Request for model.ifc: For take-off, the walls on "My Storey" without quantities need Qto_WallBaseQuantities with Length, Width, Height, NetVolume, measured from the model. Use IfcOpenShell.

First a look at what the model holds.

```python
import ifcopenshell
import ifcopenshell.util.element
import ifcopenshell.util.unit

model = ifcopenshell.open("model.ifc")
print(model.schema)
for unit_type in ("LENGTHUNIT", "AREAUNIT", "VOLUMEUNIT"):
    print(unit_type, ifcopenshell.util.unit.calculate_unit_scale(model, unit_type))
storey = next(s for s in model.by_type("IfcBuildingStorey") if s.Name == "My Storey")
walls = [e for e in ifcopenshell.util.element.get_decomposition(storey) if e.is_a("IfcWall")]
for e in sorted(walls, key=lambda e: e.id()):
    print(e.id(), e.is_a(), e.Name, list(ifcopenshell.util.element.get_psets(e, qtos_only=True)), sep=" | ")
```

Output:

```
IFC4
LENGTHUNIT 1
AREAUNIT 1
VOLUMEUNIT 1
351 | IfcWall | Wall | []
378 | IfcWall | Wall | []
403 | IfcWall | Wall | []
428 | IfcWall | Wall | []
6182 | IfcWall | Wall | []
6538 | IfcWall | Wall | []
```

```python
import ifcopenshell
import ifcopenshell.api.pset
import ifcopenshell.geom
import ifcopenshell.util.element
import ifcopenshell.util.shape
import ifcopenshell.util.unit

model = ifcopenshell.open("model.ifc")
unit_scale = ifcopenshell.util.unit.calculate_unit_scale(model)
volume_scale = ifcopenshell.util.unit.calculate_unit_scale(model, "VOLUMEUNIT")
settings = ifcopenshell.geom.settings()

storey = next(s for s in model.by_type("IfcBuildingStorey") if s.Name == "My Storey")
walls = [e for e in ifcopenshell.util.element.get_decomposition(storey) if e.is_a("IfcWall")]

for e in sorted(walls, key=lambda e: e.id()):
    if ifcopenshell.util.element.get_psets(e, qtos_only=True, should_inherit=False):
        continue
    # Geometry comes back in metres, in the element's own axes.
    shape = ifcopenshell.geom.create_shape(settings, e)
    values = {
        "Length": ifcopenshell.util.shape.get_x(shape.geometry) / unit_scale,
        "Width": ifcopenshell.util.shape.get_y(shape.geometry) / unit_scale,
        "Height": ifcopenshell.util.shape.get_z(shape.geometry) / unit_scale,
        "NetVolume": ifcopenshell.util.shape.get_volume(shape.geometry) / volume_scale,
    }
    qto = ifcopenshell.api.pset.add_qto(model, product=e, name="Qto_WallBaseQuantities")
    ifcopenshell.api.pset.edit_qto(model, qto=qto, properties=values)
    print(e.id(), {k: round(v, 3) for k, v in values.items()})

model.write("model_rev.ifc")
```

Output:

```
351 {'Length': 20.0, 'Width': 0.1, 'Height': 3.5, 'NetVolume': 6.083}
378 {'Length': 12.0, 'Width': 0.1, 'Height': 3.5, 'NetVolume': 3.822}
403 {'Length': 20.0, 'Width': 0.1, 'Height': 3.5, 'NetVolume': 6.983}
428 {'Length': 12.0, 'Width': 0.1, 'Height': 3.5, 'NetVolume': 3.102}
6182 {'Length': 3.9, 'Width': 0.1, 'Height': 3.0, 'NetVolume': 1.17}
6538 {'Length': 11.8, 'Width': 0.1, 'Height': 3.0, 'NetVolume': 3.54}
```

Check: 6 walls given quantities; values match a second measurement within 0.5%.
